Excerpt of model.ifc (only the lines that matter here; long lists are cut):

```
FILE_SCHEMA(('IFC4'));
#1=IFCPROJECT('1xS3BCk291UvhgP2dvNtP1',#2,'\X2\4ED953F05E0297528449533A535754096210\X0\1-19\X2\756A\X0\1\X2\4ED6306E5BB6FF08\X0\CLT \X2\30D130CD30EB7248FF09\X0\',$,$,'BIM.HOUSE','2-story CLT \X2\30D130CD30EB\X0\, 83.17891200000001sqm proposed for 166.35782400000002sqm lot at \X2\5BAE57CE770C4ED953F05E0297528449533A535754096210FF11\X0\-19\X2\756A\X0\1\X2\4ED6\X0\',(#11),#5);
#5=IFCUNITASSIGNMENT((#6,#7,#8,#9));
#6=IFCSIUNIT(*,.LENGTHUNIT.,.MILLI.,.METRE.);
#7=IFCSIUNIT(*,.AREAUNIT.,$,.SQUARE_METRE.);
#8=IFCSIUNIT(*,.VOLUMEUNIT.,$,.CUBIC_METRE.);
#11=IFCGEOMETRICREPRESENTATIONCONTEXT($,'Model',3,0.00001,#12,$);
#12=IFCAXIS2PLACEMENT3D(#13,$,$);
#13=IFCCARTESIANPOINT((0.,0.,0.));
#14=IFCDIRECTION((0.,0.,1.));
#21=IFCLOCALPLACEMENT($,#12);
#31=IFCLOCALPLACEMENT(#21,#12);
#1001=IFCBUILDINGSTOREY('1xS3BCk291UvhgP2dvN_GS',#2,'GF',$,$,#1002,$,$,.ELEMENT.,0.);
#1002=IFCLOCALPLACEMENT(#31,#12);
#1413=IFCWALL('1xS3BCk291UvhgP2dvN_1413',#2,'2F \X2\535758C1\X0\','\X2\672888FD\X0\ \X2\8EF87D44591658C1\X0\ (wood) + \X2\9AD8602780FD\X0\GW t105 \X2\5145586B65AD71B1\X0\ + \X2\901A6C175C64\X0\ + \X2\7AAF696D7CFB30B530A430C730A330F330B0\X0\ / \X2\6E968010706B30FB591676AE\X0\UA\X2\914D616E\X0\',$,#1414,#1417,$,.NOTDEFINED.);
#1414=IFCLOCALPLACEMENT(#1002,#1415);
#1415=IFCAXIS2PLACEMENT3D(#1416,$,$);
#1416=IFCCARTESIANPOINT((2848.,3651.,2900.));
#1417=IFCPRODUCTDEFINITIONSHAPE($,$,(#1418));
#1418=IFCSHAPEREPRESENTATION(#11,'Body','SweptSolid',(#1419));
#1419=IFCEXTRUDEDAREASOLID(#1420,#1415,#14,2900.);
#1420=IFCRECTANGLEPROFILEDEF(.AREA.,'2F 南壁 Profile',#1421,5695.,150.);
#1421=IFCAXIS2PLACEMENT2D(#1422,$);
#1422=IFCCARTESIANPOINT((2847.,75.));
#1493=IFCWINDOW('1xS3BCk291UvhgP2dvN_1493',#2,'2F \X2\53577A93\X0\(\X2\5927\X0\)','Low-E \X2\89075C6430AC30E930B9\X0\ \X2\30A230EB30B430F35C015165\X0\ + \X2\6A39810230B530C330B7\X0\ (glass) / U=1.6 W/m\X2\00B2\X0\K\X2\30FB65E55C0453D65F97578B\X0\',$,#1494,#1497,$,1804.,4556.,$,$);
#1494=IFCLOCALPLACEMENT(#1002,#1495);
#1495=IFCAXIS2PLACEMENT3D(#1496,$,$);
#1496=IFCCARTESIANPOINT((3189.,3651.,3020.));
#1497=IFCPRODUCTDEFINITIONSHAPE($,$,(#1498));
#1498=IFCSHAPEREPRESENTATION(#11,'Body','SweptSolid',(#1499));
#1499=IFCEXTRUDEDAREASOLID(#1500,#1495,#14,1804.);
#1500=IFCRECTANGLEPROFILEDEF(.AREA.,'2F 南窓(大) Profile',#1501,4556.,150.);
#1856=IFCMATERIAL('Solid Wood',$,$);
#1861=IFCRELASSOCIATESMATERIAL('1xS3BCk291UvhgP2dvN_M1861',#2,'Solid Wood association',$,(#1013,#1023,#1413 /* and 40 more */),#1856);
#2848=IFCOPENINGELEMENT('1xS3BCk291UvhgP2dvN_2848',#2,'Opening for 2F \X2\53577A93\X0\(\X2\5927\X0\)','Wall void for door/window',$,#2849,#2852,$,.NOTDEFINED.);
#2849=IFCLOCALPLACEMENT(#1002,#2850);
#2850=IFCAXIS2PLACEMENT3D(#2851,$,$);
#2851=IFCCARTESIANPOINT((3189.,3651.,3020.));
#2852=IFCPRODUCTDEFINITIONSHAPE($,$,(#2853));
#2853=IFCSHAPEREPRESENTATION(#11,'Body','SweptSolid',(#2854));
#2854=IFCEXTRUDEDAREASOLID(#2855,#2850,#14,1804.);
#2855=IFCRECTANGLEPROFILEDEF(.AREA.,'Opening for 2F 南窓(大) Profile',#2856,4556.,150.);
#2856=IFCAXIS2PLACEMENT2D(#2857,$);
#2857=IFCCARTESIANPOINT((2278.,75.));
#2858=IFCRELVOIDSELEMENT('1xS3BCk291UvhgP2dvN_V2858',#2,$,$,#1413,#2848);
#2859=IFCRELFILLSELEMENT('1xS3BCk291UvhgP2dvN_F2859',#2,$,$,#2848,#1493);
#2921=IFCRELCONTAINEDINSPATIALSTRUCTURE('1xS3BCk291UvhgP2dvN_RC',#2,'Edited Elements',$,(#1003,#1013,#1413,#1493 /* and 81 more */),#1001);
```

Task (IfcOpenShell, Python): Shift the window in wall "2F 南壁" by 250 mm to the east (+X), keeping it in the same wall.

```python
import ifcopenshell
import ifcopenshell.api.geometry
import ifcopenshell.util.placement

model = ifcopenshell.open("model.ifc")

window = model.by_id(1493)
opening = window.FillsVoids[0].RelatingOpeningElement
wall = opening.VoidsElements[0].RelatingBuildingElement

wall_matrix = ifcopenshell.util.placement.get_local_placement(wall.ObjectPlacement)
shift = wall_matrix[:3, 0] * 250.0
before = ifcopenshell.util.placement.get_local_placement(window.ObjectPlacement)[:3, 3].copy()

# The window is not placed relative to its opening, so move both.
for product in (opening, window):
    matrix = ifcopenshell.util.placement.get_local_placement(product.ObjectPlacement)
    matrix[:3, 3] += shift
    ifcopenshell.api.geometry.edit_object_placement(model, product=product, matrix=matrix, is_si=False)

after = ifcopenshell.util.placement.get_local_placement(window.ObjectPlacement)[:3, 3]
print("window moved by", (after - before).round(3) + 0.0)

model.write("model-out.ifc")
```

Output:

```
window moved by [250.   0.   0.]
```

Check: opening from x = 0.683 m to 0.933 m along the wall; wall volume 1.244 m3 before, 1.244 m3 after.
